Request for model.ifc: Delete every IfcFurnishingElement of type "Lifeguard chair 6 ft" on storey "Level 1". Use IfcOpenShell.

First a look at what the model holds.

```python
import ifcopenshell
import ifcopenshell.util.element

model = ifcopenshell.open("model.ifc")
print(model.schema)
storey = next(s for s in model.by_type("IfcBuildingStorey") if s.Name == "Level 1")
furniture = [e for e in ifcopenshell.util.element.get_decomposition(storey) if e.is_a("IfcFurnishingElement")]
seen = {}
for e in furniture:
    element_type = ifcopenshell.util.element.get_type(e)
    name = element_type.Name if element_type not in (None, e) else None
    seen[name] = seen.get(name, 0) + 1
for name, count in sorted(seen.items(), key=str):
    print(count, "x", name)
```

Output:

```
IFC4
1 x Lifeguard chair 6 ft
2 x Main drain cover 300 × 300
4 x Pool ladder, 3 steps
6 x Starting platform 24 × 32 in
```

```python
import ifcopenshell
import ifcopenshell.api.root
import ifcopenshell.util.element

model = ifcopenshell.open("model.ifc")

storey = next(s for s in model.by_type("IfcBuildingStorey") if s.Name == "Level 1")
furniture = [e for e in ifcopenshell.util.element.get_decomposition(storey) if e.is_a("IfcFurnishingElement")]
targets = [e for e in furniture if (t := ifcopenshell.util.element.get_type(e)) not in (None, e) and t.Name == "Lifeguard chair 6 ft"]

for e in targets:
    ifcopenshell.api.root.remove_product(model, product=e)
print(len(targets), "removed")

model.write("model_edited.ifc")
```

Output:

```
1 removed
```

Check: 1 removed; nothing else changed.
